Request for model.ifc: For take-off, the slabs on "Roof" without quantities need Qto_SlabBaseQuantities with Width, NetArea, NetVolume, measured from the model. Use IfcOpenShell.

First a look at what the model holds.

```python
import ifcopenshell
import ifcopenshell.util.element
import ifcopenshell.util.unit

model = ifcopenshell.open("model.ifc")
print(model.schema)
for unit_type in ("LENGTHUNIT", "AREAUNIT", "VOLUMEUNIT"):
    print(unit_type, ifcopenshell.util.unit.calculate_unit_scale(model, unit_type))
storey = next(s for s in model.by_type("IfcBuildingStorey") if s.Name == "Roof")
slabs = [e for e in ifcopenshell.util.element.get_decomposition(storey) if e.is_a("IfcSlab")]
for e in sorted(slabs, key=lambda e: e.id()):
    print(e.id(), e.is_a(), e.Name, list(ifcopenshell.util.element.get_psets(e, qtos_only=True)), sep=" | ")
```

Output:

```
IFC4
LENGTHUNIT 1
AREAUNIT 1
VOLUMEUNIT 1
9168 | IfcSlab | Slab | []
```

```python
import ifcopenshell
import ifcopenshell.api.pset
import ifcopenshell.geom
import ifcopenshell.util.element
import ifcopenshell.util.shape
import ifcopenshell.util.unit

model = ifcopenshell.open("model.ifc")
unit_scale = ifcopenshell.util.unit.calculate_unit_scale(model)
area_scale = ifcopenshell.util.unit.calculate_unit_scale(model, "AREAUNIT")
volume_scale = ifcopenshell.util.unit.calculate_unit_scale(model, "VOLUMEUNIT")
settings = ifcopenshell.geom.settings()

storey = next(s for s in model.by_type("IfcBuildingStorey") if s.Name == "Roof")
slabs = [e for e in ifcopenshell.util.element.get_decomposition(storey) if e.is_a("IfcSlab")]

for e in sorted(slabs, key=lambda e: e.id()):
    if ifcopenshell.util.element.get_psets(e, qtos_only=True, should_inherit=False):
        continue
    # Geometry comes back in metres, in the element's own axes.
    shape = ifcopenshell.geom.create_shape(settings, e)
    values = {
        "Width": ifcopenshell.util.shape.get_z(shape.geometry) / unit_scale,
        "NetArea": ifcopenshell.util.shape.get_footprint_area(shape.geometry) / area_scale,
        "NetVolume": ifcopenshell.util.shape.get_volume(shape.geometry) / volume_scale,
    }
    qto = ifcopenshell.api.pset.add_qto(model, product=e, name="Qto_SlabBaseQuantities")
    ifcopenshell.api.pset.edit_qto(model, qto=qto, properties=values)
    print(e.id(), {k: round(v, 3) for k, v in values.items()})

model.write("model_edited.ifc")
```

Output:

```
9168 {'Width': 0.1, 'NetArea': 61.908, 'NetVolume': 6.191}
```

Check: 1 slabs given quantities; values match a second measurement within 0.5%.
